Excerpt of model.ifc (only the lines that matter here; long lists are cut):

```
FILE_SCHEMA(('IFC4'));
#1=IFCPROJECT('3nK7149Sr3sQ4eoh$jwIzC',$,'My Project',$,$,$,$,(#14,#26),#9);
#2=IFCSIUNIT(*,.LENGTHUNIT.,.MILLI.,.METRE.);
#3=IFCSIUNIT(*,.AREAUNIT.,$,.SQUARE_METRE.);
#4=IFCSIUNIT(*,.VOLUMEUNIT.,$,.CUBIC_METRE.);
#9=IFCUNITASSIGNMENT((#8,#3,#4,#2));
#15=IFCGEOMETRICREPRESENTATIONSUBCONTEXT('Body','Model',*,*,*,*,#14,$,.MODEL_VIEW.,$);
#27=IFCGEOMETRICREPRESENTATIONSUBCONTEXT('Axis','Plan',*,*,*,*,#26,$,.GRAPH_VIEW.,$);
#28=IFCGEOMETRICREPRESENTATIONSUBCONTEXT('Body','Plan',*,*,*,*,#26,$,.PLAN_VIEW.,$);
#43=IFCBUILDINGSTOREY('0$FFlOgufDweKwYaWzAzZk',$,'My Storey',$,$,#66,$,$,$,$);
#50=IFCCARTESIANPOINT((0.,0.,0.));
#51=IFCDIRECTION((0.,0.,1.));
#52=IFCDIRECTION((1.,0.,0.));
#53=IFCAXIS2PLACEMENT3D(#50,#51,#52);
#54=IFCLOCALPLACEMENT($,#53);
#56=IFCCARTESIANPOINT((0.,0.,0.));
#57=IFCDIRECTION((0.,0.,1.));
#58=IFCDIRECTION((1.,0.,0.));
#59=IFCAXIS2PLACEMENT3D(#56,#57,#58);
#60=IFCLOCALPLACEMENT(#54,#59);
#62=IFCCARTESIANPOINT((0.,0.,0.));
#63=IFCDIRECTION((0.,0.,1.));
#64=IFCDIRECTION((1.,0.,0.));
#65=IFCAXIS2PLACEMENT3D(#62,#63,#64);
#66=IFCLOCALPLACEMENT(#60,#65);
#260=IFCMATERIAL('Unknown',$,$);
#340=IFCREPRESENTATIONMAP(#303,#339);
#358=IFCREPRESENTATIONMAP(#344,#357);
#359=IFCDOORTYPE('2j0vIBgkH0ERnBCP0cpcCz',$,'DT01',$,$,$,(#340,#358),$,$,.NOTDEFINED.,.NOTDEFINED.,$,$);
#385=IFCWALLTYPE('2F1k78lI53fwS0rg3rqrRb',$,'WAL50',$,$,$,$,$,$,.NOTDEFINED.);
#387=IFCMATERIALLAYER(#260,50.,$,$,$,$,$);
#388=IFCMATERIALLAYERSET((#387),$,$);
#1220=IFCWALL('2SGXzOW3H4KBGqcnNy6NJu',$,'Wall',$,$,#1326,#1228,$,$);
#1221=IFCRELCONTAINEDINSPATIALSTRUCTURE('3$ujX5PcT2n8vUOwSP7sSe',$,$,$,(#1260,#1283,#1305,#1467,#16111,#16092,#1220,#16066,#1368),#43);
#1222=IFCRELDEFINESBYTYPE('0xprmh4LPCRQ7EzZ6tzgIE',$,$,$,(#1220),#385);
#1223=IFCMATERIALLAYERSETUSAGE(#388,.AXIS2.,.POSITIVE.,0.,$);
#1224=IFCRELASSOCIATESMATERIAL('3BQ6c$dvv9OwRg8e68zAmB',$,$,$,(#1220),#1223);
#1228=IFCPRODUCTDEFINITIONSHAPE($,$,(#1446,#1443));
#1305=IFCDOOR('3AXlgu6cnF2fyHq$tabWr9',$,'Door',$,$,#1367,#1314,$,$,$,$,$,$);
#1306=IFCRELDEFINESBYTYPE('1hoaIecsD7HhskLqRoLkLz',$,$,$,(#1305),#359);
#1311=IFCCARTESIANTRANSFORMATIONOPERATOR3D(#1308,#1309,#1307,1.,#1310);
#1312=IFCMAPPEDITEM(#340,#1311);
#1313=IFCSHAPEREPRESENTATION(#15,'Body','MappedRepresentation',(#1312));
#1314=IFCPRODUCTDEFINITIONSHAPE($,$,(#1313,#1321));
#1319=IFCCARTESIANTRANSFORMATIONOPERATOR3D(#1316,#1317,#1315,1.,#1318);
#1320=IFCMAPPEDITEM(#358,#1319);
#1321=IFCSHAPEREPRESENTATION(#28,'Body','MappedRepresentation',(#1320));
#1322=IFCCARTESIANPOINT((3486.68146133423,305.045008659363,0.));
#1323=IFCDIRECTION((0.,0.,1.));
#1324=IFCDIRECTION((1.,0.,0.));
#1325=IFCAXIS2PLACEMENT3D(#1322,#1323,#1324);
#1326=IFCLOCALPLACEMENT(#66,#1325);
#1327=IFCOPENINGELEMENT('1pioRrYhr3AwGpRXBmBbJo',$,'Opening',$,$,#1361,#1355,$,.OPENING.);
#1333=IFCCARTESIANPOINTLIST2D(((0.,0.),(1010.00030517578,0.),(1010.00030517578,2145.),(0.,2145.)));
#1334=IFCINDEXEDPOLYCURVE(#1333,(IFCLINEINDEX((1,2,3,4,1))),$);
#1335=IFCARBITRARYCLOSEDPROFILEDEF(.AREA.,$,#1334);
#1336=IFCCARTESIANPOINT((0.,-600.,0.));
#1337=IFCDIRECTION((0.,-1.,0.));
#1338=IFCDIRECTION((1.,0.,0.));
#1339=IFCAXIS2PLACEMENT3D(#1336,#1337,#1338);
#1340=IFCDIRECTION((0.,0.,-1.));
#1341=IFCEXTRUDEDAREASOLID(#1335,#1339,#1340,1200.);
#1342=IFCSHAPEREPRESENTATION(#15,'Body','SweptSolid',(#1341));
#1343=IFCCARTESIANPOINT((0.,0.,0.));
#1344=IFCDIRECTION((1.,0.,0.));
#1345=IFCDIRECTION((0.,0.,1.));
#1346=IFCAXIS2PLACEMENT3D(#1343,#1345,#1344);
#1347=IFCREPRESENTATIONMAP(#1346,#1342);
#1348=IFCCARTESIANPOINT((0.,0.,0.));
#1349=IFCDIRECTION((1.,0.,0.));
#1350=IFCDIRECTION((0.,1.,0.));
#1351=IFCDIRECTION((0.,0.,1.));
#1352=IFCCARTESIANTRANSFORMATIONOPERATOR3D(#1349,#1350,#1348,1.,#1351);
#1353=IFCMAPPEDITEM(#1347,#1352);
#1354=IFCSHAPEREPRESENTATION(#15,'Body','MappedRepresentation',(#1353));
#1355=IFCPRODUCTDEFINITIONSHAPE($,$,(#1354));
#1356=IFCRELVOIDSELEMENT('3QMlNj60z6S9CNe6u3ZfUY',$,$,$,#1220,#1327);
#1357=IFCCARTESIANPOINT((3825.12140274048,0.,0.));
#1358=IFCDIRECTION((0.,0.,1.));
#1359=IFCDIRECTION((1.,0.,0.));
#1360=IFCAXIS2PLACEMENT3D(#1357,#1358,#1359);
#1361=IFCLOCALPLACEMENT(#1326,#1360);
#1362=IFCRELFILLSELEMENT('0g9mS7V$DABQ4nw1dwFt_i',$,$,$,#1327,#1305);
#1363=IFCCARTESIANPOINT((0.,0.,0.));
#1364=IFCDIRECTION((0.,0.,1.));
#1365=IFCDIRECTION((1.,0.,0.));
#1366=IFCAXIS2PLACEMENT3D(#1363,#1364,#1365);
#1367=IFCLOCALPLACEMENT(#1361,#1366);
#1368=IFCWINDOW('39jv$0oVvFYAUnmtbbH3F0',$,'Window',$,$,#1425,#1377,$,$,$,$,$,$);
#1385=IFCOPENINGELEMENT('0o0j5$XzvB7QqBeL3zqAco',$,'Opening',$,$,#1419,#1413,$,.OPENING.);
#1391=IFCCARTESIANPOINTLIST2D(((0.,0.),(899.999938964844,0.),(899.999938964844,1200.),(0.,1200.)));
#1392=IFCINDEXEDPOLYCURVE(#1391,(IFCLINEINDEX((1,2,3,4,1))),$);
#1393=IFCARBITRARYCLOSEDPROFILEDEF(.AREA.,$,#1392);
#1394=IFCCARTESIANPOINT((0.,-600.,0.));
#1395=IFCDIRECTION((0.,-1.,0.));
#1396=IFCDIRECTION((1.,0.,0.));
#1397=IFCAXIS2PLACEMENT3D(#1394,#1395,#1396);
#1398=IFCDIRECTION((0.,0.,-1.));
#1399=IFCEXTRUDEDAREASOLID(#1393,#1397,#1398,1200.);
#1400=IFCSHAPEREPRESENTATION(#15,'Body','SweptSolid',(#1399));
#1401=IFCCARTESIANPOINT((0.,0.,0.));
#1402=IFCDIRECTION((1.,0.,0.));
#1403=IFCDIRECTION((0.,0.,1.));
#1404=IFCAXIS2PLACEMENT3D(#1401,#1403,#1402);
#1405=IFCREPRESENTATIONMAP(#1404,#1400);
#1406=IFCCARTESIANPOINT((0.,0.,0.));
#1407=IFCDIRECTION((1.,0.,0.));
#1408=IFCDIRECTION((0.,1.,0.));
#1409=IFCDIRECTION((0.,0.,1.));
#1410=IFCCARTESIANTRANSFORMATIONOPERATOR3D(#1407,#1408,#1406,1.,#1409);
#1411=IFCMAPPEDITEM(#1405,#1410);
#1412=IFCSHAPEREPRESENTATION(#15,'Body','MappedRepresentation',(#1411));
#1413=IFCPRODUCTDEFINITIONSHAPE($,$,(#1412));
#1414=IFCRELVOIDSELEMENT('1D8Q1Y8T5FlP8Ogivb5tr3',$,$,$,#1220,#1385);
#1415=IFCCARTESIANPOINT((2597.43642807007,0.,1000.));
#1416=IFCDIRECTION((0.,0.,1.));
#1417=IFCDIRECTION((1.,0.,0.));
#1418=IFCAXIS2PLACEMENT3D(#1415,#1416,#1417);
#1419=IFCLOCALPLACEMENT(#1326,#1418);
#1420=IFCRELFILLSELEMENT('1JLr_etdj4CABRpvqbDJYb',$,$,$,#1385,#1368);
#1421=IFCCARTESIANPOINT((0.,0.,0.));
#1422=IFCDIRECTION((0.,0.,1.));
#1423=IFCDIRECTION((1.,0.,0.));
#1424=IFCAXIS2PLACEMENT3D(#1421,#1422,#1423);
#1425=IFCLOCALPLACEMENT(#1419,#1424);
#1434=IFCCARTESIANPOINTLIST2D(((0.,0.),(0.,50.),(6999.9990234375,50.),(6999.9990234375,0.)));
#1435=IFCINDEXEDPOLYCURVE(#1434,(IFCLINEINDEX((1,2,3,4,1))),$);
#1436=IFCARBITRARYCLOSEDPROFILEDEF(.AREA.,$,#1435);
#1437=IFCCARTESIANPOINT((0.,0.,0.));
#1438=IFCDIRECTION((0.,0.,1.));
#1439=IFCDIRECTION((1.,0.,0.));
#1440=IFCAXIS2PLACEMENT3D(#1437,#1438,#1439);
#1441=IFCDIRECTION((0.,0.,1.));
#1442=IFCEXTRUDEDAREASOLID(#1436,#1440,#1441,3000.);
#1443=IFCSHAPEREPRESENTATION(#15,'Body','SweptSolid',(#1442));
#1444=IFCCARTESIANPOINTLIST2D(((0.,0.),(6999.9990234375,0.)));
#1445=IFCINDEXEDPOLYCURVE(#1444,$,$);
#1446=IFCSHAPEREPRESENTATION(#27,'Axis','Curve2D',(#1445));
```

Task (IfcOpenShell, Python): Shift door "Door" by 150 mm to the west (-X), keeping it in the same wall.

```python
import ifcopenshell
import ifcopenshell.api.geometry
import ifcopenshell.util.placement
import ifcopenshell.util.unit

model = ifcopenshell.open("model.ifc")
unit_scale = ifcopenshell.util.unit.calculate_unit_scale(model)

door = model.by_id(1305)
opening = door.FillsVoids[0].RelatingOpeningElement
wall = opening.VoidsElements[0].RelatingBuildingElement

wall_matrix = ifcopenshell.util.placement.get_local_placement(wall.ObjectPlacement)
shift = wall_matrix[:3, 0] * -0.15 / unit_scale
before = ifcopenshell.util.placement.get_local_placement(door.ObjectPlacement)[:3, 3].copy()

# The door is placed relative to its opening, so it follows when the opening moves.
matrix = ifcopenshell.util.placement.get_local_placement(opening.ObjectPlacement)
matrix[:3, 3] += shift
ifcopenshell.api.geometry.edit_object_placement(
    model, product=opening, matrix=matrix, is_si=False, should_transform_children=True
)

after = ifcopenshell.util.placement.get_local_placement(door.ObjectPlacement)[:3, 3]
print("door moved by", (after - before).round(3) + 0.0)

model.write("model_v2.ifc")
```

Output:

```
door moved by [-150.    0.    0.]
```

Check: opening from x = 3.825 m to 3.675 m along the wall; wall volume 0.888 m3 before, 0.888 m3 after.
